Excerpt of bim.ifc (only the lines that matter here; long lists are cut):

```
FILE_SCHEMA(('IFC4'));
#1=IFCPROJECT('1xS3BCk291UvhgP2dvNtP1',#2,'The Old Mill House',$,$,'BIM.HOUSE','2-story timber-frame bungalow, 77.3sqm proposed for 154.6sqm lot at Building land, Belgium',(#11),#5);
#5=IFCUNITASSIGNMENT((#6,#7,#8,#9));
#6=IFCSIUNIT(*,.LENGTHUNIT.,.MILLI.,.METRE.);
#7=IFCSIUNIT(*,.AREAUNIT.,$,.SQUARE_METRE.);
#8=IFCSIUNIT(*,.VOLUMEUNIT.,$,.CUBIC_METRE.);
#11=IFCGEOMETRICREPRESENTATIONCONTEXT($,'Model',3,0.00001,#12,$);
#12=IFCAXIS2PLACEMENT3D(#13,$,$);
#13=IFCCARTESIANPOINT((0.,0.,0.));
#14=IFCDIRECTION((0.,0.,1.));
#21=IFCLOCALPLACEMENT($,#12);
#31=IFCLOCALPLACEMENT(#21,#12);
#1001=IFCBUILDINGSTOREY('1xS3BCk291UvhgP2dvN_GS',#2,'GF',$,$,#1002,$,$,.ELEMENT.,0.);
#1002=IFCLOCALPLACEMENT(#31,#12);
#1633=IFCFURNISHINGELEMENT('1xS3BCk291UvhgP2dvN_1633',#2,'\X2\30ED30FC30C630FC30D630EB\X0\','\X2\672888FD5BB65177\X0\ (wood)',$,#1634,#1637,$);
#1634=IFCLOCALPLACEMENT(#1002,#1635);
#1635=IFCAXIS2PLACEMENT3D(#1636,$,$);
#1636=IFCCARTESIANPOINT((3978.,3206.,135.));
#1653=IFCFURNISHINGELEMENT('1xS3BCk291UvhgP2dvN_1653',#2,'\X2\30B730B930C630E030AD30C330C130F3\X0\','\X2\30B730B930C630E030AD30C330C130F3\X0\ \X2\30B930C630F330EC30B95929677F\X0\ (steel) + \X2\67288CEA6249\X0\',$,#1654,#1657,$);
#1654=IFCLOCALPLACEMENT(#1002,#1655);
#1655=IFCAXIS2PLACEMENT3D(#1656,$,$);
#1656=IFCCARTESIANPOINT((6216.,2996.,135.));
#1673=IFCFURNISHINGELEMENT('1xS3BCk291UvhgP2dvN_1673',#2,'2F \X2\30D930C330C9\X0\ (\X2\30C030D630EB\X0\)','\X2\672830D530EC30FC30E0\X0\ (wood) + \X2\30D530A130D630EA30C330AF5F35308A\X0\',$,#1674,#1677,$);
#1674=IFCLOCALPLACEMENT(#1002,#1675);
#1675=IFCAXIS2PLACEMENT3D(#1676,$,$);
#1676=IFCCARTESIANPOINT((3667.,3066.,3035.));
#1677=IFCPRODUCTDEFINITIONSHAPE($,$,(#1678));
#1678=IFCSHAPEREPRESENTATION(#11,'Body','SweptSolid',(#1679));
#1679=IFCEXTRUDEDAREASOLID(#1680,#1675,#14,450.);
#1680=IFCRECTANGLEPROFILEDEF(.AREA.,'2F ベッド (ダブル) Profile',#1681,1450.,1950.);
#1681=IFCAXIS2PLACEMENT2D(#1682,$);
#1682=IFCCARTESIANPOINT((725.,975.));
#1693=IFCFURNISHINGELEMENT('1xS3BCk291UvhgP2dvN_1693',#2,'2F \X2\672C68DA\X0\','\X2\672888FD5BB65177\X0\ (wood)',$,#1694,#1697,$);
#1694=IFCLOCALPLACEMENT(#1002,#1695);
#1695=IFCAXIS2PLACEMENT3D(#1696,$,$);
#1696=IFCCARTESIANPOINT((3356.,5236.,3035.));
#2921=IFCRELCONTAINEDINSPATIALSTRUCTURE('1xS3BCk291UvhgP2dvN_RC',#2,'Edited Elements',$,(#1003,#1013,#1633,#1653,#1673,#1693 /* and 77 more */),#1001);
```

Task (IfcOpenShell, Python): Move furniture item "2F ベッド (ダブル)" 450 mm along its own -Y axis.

```python
import ifcopenshell
import ifcopenshell.api.geometry
import ifcopenshell.util.placement
import ifcopenshell.util.unit

model = ifcopenshell.open("bim.ifc")
unit_scale = ifcopenshell.util.unit.calculate_unit_scale(model)

item = model.by_id(1673)
matrix = ifcopenshell.util.placement.get_local_placement(item.ObjectPlacement)
matrix[:3, 3] -= matrix[:3, 1] * 0.45 / unit_scale
ifcopenshell.api.geometry.edit_object_placement(model, product=item, matrix=matrix, is_si=False)

print(ifcopenshell.util.placement.get_local_placement(item.ObjectPlacement).round(3) + 0.0)

model.write("bim_edited.ifc")
```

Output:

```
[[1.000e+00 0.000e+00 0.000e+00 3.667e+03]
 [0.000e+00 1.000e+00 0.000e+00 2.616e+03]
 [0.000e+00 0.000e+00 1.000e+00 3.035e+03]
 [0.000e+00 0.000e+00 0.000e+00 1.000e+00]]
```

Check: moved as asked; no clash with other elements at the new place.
